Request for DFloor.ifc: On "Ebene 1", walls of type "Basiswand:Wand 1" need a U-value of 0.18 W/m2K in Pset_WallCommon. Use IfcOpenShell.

First a look at what the model holds.

```python
import ifcopenshell
import ifcopenshell.util.element

model = ifcopenshell.open("DFloor.ifc")
print(model.schema)
storey = next(s for s in model.by_type("IfcBuildingStorey") if s.Name == "Ebene 1")
walls = [e for e in ifcopenshell.util.element.get_decomposition(storey) if e.is_a("IfcWall")]
seen = {}
for e in walls:
    element_type = ifcopenshell.util.element.get_type(e)
    key = (element_type.Name if element_type != e and element_type else None, ifcopenshell.util.element.get_pset(e, "Pset_WallCommon", "ThermalTransmittance"))
    seen[key] = seen.get(key, 0) + 1
for (name, value), count in sorted(seen.items(), key=str):
    print(count, "x", name, "|", value)
```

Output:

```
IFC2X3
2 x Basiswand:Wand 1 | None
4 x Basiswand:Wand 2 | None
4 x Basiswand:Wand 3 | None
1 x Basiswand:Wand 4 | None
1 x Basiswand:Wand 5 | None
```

```python
import ifcopenshell
import ifcopenshell.api.pset
import ifcopenshell.util.element

model = ifcopenshell.open("DFloor.ifc")

storey = next(s for s in model.by_type("IfcBuildingStorey") if s.Name == "Ebene 1")
walls = [e for e in ifcopenshell.util.element.get_decomposition(storey) if e.is_a("IfcWall")]

count = 0
for e in walls:
    element_type = ifcopenshell.util.element.get_type(e)
    if element_type in (None, e) or element_type.Name != "Basiswand:Wand 1":
        continue
    # add_pset returns the element's existing set when there is one.
    pset = ifcopenshell.api.pset.add_pset(model, product=e, name="Pset_WallCommon")
    ifcopenshell.api.pset.edit_pset(model, pset=pset, properties={"ThermalTransmittance": 0.18})
    count += 1

print(count, "walls updated")

model.write("DFloor_updated.ifc")
```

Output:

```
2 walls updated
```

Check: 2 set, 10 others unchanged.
